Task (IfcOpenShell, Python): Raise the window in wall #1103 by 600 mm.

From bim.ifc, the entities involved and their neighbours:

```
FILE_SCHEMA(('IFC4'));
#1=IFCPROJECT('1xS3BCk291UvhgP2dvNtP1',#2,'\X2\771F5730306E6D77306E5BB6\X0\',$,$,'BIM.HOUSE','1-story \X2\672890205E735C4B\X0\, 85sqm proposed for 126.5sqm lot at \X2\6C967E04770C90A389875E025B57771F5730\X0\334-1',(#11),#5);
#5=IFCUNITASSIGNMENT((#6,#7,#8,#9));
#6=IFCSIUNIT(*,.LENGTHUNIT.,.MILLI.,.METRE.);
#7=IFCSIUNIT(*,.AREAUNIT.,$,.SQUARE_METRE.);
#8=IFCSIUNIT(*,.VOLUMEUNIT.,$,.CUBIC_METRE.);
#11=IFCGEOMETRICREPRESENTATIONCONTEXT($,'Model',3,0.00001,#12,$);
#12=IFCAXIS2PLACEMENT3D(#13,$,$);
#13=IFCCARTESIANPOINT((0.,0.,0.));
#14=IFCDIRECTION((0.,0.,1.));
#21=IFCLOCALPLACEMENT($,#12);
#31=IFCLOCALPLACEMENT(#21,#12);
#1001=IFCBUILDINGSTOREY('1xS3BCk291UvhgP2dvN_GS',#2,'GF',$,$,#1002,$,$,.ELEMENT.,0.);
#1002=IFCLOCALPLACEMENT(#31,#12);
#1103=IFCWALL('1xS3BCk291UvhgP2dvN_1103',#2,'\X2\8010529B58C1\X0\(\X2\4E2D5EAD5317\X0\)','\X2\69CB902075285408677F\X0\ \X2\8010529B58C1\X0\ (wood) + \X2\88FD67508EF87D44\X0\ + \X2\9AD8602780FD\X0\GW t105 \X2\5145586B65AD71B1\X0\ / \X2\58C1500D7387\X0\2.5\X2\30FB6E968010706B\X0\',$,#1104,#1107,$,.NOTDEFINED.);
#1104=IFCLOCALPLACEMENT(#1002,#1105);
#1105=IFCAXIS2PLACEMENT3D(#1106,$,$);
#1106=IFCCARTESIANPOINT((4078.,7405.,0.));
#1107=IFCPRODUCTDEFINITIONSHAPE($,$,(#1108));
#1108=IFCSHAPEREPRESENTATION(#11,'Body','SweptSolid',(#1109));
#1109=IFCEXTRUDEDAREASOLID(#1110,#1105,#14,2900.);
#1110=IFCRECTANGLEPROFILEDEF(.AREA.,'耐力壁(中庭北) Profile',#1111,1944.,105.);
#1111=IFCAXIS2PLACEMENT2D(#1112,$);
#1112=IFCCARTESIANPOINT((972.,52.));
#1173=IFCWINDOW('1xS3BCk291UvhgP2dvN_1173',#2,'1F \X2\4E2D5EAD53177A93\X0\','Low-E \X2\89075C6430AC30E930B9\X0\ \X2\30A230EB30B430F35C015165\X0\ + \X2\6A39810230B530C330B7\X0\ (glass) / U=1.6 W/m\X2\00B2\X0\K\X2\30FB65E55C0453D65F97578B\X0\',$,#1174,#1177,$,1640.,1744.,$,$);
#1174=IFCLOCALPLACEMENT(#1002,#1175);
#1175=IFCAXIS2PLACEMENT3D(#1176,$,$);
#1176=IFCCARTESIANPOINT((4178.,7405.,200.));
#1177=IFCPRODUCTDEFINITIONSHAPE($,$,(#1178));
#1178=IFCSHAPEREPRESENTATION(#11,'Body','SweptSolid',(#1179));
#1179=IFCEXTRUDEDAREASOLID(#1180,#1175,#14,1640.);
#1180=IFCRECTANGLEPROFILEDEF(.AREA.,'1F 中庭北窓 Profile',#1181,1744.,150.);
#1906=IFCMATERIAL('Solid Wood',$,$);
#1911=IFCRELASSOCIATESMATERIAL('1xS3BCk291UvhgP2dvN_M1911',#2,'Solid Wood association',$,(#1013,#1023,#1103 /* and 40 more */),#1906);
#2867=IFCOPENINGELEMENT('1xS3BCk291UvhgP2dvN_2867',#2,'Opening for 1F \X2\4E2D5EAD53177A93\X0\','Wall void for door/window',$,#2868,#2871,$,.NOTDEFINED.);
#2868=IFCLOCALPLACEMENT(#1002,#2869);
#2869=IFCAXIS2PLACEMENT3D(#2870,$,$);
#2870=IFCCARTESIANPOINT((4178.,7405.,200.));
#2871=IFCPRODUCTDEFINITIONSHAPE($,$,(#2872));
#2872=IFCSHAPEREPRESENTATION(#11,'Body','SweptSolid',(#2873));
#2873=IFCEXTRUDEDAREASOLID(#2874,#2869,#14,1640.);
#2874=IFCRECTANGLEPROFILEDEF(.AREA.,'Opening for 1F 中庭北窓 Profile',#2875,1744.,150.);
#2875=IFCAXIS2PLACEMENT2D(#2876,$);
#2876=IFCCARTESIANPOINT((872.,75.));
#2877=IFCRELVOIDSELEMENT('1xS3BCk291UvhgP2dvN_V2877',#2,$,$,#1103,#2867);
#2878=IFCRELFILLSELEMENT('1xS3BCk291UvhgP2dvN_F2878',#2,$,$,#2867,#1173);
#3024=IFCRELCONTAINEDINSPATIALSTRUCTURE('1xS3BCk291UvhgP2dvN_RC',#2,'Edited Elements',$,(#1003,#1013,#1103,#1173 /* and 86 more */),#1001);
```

```python
import numpy as np
import ifcopenshell
import ifcopenshell.api.geometry
import ifcopenshell.util.placement
import ifcopenshell.util.unit

model = ifcopenshell.open("bim.ifc")
unit_scale = ifcopenshell.util.unit.calculate_unit_scale(model)

window = model.by_guid("1xS3BCk291UvhgP2dvN_1173")
opening = window.FillsVoids[0].RelatingOpeningElement
dz = 0.6 / unit_scale

shift = np.array([0.0, 0.0, dz])
# The window is not placed relative to its opening, so move both.
for product in (opening, window):
    matrix = ifcopenshell.util.placement.get_local_placement(product.ObjectPlacement)
    matrix[:3, 3] += shift
    ifcopenshell.api.geometry.edit_object_placement(model, product=product, matrix=matrix, is_si=False)

print(f"moved by {dz * unit_scale:+.3f} m")

model.write("bim_edited.ifc")
```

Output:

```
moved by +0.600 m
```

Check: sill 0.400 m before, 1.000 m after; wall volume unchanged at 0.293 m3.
